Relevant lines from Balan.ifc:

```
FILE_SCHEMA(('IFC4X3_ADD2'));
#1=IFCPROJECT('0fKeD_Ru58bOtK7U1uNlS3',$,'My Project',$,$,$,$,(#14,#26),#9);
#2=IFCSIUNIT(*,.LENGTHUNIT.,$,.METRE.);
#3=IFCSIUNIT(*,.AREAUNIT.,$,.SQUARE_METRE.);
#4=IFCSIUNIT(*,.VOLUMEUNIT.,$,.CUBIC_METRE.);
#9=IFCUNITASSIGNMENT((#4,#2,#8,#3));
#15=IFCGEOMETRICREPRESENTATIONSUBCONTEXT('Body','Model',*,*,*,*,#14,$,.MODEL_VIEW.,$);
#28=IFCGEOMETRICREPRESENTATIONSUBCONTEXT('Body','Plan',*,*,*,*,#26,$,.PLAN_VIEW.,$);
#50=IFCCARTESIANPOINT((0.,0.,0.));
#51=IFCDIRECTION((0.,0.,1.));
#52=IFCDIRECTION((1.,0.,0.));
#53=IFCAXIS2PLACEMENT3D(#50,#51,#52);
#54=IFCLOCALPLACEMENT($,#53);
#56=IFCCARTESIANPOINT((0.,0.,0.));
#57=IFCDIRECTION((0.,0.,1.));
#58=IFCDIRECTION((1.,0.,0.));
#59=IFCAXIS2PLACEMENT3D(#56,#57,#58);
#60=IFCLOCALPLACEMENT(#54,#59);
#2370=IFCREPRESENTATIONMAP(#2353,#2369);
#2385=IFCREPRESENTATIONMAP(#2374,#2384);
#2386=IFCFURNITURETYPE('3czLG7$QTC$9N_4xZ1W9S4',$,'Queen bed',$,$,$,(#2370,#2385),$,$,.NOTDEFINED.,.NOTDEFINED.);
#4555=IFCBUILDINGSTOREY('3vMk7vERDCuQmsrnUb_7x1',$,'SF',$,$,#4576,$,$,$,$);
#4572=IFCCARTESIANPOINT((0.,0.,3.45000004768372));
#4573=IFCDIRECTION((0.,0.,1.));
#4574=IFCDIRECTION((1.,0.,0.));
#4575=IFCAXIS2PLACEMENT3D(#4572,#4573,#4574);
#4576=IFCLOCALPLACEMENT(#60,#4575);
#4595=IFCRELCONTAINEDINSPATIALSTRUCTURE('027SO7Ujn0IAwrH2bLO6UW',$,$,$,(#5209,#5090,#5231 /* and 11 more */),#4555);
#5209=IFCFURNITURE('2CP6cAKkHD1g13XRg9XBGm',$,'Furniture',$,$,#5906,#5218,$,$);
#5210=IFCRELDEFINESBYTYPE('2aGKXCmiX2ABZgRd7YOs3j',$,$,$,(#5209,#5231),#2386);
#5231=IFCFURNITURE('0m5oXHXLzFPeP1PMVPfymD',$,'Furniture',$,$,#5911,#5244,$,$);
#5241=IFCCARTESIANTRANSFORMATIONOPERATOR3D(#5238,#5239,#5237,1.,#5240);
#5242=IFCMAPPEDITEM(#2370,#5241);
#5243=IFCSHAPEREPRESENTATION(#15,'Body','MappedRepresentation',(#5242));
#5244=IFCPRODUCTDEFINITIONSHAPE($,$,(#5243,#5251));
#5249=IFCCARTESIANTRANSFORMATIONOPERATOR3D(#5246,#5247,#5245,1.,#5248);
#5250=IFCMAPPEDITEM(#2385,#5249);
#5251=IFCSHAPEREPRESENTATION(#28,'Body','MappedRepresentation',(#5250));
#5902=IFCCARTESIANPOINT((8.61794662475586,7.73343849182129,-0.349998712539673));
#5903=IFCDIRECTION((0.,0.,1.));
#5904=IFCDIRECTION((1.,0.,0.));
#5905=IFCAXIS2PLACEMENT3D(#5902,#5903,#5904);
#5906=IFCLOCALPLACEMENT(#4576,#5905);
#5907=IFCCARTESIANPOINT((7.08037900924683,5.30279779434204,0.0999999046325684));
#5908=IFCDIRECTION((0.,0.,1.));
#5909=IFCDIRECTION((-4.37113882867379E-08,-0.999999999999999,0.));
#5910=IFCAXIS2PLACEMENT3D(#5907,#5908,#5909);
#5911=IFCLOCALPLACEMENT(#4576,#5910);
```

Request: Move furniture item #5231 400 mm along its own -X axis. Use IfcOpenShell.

```python
import ifcopenshell
import ifcopenshell.api.geometry
import ifcopenshell.util.placement
import ifcopenshell.util.unit

model = ifcopenshell.open("Balan.ifc")
unit_scale = ifcopenshell.util.unit.calculate_unit_scale(model)

item = model.by_guid("0m5oXHXLzFPeP1PMVPfymD")
matrix = ifcopenshell.util.placement.get_local_placement(item.ObjectPlacement)
matrix[:3, 3] -= matrix[:3, 0] * 0.4 / unit_scale
ifcopenshell.api.geometry.edit_object_placement(model, product=item, matrix=matrix, is_si=False)

print(ifcopenshell.util.placement.get_local_placement(item.ObjectPlacement).round(3) + 0.0)

model.write("Balan_rev.ifc")
```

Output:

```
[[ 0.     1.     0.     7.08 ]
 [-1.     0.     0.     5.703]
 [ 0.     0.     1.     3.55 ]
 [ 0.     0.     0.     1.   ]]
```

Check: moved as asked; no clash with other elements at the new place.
